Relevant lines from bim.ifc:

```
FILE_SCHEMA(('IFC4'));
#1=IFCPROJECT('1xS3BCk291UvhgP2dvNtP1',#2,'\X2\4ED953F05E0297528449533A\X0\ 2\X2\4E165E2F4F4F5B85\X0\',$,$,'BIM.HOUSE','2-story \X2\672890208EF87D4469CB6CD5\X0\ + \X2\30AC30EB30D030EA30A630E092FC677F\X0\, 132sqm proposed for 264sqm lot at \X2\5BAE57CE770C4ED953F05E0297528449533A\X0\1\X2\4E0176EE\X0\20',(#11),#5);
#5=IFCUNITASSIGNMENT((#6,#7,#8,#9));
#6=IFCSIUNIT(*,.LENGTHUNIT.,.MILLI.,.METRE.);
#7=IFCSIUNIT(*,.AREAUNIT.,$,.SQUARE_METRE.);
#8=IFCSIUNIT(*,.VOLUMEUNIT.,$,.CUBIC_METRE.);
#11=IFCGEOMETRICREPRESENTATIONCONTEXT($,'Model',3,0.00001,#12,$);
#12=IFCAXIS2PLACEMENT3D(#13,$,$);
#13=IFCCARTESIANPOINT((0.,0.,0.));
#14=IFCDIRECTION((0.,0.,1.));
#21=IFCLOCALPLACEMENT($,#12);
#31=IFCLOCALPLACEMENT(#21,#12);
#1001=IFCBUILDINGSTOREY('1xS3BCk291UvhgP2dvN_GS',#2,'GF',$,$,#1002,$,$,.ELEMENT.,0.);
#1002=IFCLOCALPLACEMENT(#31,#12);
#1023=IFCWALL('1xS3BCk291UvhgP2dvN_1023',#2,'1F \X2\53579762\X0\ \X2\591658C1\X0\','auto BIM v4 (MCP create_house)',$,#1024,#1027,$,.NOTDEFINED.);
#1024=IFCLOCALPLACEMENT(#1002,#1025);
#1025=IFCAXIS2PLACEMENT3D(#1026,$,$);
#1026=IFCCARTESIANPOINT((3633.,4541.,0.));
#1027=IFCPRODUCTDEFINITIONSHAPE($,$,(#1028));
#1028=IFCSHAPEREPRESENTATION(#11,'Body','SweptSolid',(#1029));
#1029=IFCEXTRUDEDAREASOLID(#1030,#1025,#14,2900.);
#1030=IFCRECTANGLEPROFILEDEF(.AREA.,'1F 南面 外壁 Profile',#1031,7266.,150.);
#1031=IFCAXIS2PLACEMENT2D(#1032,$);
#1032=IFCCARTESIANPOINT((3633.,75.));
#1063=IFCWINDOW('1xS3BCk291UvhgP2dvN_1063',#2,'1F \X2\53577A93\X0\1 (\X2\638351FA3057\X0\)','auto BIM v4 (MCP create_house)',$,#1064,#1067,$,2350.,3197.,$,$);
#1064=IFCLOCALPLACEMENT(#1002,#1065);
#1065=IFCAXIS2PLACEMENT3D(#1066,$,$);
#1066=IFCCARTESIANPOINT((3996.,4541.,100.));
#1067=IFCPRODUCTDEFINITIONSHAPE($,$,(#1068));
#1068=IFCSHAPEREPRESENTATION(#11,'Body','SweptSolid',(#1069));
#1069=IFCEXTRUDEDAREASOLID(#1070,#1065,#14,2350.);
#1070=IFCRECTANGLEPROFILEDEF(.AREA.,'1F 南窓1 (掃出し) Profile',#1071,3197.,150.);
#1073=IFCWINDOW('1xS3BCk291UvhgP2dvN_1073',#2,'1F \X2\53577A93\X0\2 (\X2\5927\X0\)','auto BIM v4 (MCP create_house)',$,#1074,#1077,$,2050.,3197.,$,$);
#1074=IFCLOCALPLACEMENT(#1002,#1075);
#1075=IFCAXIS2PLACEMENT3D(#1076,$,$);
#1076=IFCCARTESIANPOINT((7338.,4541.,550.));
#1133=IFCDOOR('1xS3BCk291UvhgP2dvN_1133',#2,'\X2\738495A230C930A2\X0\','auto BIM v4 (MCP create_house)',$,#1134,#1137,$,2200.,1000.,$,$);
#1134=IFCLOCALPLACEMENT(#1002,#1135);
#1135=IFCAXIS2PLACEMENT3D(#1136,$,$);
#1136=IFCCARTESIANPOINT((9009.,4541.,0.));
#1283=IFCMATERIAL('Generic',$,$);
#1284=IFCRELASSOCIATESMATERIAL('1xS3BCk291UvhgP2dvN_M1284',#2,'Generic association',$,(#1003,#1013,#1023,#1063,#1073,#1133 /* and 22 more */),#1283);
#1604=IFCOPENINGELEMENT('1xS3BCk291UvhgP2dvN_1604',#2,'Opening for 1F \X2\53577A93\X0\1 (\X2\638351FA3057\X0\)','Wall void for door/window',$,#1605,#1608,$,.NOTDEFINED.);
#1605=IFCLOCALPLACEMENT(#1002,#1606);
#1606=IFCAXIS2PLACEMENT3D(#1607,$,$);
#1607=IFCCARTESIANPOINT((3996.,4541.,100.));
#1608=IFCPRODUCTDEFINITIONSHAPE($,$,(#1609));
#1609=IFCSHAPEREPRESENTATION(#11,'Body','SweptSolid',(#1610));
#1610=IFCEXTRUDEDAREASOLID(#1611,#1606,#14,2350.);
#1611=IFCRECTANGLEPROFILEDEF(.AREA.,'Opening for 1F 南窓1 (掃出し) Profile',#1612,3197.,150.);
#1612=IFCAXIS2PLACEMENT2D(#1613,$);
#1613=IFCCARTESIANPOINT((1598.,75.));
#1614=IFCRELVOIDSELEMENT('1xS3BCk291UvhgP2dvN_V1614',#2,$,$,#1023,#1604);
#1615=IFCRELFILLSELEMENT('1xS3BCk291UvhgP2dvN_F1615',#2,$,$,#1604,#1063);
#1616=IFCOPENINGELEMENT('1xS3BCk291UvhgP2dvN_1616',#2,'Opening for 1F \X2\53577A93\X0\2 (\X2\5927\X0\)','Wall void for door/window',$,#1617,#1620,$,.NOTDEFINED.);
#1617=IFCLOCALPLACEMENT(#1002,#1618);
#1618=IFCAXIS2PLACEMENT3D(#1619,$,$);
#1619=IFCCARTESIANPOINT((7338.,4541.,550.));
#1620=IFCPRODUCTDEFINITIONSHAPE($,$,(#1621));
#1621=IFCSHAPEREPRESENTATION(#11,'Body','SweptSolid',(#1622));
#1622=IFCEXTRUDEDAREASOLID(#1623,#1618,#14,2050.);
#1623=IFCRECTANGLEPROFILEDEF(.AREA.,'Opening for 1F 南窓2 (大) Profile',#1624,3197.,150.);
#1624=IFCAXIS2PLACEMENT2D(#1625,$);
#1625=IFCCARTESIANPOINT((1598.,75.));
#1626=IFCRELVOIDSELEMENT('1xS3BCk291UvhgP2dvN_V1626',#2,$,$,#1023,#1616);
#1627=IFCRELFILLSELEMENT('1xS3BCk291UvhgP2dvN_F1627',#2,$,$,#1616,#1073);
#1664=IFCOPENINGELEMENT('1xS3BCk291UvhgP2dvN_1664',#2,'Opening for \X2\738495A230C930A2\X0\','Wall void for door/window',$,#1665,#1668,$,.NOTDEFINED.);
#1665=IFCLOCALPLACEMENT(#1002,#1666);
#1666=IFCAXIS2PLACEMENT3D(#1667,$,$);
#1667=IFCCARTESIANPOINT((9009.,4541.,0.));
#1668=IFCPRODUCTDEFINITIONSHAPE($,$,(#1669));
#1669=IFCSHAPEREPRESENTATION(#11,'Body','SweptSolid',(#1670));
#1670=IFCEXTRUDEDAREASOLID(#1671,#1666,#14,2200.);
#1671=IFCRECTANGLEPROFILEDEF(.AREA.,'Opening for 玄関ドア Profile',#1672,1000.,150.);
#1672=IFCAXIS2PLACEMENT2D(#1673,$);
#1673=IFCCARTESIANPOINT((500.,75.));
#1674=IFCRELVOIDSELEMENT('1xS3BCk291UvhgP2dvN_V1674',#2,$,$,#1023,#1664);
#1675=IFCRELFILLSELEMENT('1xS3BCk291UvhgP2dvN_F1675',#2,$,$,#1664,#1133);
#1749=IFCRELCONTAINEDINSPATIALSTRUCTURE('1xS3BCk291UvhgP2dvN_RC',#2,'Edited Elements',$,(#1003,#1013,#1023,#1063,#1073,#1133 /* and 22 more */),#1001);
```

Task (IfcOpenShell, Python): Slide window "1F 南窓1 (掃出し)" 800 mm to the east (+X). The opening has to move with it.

```python
import ifcopenshell
import ifcopenshell.api.geometry
import ifcopenshell.util.placement
import ifcopenshell.util.unit

model = ifcopenshell.open("bim.ifc")
unit_scale = ifcopenshell.util.unit.calculate_unit_scale(model)

window = model.by_guid("1xS3BCk291UvhgP2dvN_1063")
opening = window.FillsVoids[0].RelatingOpeningElement
wall = opening.VoidsElements[0].RelatingBuildingElement

wall_matrix = ifcopenshell.util.placement.get_local_placement(wall.ObjectPlacement)
shift = wall_matrix[:3, 0] * 0.8 / unit_scale
before = ifcopenshell.util.placement.get_local_placement(window.ObjectPlacement)[:3, 3].copy()

# The window is not placed relative to its opening, so move both.
for product in (opening, window):
    matrix = ifcopenshell.util.placement.get_local_placement(product.ObjectPlacement)
    matrix[:3, 3] += shift
    ifcopenshell.api.geometry.edit_object_placement(model, product=product, matrix=matrix, is_si=False)

after = ifcopenshell.util.placement.get_local_placement(window.ObjectPlacement)[:3, 3]
print("window moved by", (after - before).round(3) + 0.0)

model.write("bim-out.ifc")
```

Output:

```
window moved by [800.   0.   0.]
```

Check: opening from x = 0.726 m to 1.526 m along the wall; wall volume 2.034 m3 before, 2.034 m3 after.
